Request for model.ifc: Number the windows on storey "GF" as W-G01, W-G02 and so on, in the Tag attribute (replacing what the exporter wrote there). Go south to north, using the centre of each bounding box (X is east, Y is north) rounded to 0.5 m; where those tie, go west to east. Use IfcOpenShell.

First a look at what the model holds.

```python
import ifcopenshell
import ifcopenshell.util.element
import ifcopenshell.util.placement

model = ifcopenshell.open("model.ifc")
print(model.schema)
storey = next(s for s in model.by_type("IfcBuildingStorey") if s.Name == "GF")
windows = [e for e in ifcopenshell.util.element.get_decomposition(storey) if e.is_a("IfcWindow")]
for e in sorted(windows, key=lambda e: e.id()):
    origin = ifcopenshell.util.placement.get_local_placement(e.ObjectPlacement)[:3, 3]
    print(e.id(), e.Tag, e.Name, origin.round(2) + 0.0, sep=" | ")
```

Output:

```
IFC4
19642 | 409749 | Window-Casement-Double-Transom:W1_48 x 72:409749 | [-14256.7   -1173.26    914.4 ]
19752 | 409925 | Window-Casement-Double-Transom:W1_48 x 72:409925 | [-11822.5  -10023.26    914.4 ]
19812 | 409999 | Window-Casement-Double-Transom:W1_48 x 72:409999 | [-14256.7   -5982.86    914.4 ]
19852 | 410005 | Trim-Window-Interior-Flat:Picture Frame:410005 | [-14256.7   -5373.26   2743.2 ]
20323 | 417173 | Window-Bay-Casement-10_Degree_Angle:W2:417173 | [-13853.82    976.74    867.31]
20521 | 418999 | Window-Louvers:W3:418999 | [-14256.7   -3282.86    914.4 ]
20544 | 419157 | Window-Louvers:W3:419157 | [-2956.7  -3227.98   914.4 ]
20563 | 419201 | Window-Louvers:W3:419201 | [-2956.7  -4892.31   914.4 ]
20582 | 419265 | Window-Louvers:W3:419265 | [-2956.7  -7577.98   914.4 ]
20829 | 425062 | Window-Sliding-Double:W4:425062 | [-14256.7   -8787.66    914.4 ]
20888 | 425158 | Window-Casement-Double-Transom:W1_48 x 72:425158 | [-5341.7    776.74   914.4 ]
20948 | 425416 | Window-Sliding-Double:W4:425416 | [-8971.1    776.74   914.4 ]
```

```python
import ifcopenshell
import ifcopenshell.geom
import ifcopenshell.util.element
import ifcopenshell.util.shape

model = ifcopenshell.open("model.ifc")
settings = ifcopenshell.geom.settings()
settings.set("use-world-coords", True)


def centre(element):
    shape = ifcopenshell.geom.create_shape(settings, element)
    return ifcopenshell.util.shape.get_bbox_centroid(shape.geometry)


storey = next(s for s in model.by_type("IfcBuildingStorey") if s.Name == "GF")
windows = [e for e in ifcopenshell.util.element.get_decomposition(storey) if e.is_a("IfcWindow")]

# Insertion points can sit at a corner or the storey origin, so sort by the geometry (in metres).
centres = {e: centre(e) for e in windows}
windows.sort(key=lambda e: (round(centres[e][1] / 0.5), centres[e][0]))

for i, e in enumerate(windows, start=1):
    number = f"W-G{i:02d}"
    e.Tag = number
    print(e.id(), number)

model.write("model_v2.ifc")
```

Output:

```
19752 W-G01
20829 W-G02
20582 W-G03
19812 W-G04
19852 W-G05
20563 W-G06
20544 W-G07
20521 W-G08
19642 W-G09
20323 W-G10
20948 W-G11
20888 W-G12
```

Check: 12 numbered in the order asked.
